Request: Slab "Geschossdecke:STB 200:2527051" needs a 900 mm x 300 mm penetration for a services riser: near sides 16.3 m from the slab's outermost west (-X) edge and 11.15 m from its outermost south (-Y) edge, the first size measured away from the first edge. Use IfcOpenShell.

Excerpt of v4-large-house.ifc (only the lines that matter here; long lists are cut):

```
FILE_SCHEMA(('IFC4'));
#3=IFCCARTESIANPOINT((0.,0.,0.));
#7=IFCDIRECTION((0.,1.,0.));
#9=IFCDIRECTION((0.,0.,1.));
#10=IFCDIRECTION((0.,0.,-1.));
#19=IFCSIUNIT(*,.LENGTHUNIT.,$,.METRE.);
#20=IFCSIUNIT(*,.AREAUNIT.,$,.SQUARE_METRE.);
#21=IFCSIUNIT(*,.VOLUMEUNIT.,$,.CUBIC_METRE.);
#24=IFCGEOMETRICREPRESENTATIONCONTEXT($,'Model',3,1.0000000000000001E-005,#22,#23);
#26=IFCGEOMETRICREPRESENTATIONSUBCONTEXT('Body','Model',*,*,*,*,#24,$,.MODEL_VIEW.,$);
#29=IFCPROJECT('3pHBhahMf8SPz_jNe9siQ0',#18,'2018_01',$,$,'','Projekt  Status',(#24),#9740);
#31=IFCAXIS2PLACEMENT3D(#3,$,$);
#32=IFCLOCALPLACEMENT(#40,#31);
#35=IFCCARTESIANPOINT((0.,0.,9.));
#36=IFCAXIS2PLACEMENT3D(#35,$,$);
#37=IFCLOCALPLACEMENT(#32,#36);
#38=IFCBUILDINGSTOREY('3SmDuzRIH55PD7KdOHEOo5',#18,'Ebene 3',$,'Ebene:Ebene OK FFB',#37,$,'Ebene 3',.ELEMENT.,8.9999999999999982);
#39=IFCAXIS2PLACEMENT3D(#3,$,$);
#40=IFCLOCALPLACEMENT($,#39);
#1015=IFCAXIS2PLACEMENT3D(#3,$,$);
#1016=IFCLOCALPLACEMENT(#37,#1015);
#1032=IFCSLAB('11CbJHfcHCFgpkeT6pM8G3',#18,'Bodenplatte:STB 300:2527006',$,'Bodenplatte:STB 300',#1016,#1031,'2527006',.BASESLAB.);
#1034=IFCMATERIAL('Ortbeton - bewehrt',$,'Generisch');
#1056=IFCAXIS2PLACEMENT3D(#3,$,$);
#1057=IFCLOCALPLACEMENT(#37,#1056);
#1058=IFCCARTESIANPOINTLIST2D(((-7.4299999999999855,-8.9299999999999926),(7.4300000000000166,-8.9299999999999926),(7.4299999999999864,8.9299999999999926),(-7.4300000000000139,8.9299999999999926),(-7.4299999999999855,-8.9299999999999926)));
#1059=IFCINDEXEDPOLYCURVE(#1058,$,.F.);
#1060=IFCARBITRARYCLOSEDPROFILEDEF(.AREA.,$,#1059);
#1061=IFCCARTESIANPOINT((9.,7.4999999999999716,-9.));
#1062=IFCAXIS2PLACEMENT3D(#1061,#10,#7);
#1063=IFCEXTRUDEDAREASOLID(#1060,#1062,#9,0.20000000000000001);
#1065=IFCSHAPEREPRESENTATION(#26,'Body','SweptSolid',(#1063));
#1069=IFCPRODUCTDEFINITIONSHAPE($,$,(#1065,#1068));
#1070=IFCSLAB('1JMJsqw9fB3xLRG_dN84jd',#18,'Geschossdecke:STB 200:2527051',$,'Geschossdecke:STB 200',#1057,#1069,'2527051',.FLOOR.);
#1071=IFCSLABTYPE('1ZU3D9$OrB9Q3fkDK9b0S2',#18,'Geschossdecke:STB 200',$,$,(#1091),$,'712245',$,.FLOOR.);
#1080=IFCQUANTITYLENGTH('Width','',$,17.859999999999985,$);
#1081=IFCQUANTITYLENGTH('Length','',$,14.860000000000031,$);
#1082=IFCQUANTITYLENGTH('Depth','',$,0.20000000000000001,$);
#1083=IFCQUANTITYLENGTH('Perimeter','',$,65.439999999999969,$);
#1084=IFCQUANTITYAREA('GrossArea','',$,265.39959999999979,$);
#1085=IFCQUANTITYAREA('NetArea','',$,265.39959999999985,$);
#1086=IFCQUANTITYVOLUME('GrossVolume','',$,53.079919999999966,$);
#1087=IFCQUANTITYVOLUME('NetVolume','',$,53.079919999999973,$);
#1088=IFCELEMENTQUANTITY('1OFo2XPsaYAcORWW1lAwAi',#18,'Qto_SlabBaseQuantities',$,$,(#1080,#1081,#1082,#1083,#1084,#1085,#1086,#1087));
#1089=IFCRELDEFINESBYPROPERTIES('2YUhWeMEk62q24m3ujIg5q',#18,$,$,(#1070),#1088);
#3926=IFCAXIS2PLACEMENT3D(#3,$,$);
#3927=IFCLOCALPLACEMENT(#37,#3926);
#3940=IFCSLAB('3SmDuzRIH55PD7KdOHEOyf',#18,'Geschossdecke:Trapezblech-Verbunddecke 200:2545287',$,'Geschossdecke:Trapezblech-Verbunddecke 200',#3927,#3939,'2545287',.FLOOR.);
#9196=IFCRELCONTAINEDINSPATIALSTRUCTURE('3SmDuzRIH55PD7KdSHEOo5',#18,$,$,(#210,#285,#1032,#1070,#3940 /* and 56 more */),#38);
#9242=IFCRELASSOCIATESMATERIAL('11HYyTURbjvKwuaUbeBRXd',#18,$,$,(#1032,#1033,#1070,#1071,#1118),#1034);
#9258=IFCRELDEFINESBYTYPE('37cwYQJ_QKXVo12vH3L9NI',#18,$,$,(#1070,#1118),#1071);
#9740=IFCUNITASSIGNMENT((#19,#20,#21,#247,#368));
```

```python
import numpy as np
import ifcopenshell
import ifcopenshell.api.feature
import ifcopenshell.api.geometry
import ifcopenshell.api.pset
import ifcopenshell.api.root
import ifcopenshell.geom
import ifcopenshell.util.element
import ifcopenshell.util.placement
import ifcopenshell.util.representation
import ifcopenshell.util.shape
import ifcopenshell.util.unit

model = ifcopenshell.open("v4-large-house.ifc")
unit_scale = ifcopenshell.util.unit.calculate_unit_scale(model)
area_scale = ifcopenshell.util.unit.calculate_unit_scale(model, "AREAUNIT")
volume_scale = ifcopenshell.util.unit.calculate_unit_scale(model, "VOLUMEUNIT")
settings = ifcopenshell.geom.settings()


def volume(element):
    """Net volume in cubic metres, openings subtracted."""
    shape = ifcopenshell.geom.create_shape(settings, element)
    return ifcopenshell.util.shape.get_volume(shape.geometry)


slab = model.by_guid("1JMJsqw9fB3xLRG_dN84jd")
before = volume(slab)

# Extent in the slab's own axes, in metres. The edges named are its -X and -Y sides.
slab_shape = ifcopenshell.geom.create_shape(settings, slab)
vertices = ifcopenshell.util.shape.get_vertices(slab_shape.geometry)
x_min, y_min, bottom = vertices.min(axis=0)
top = vertices[:, 2].max()

opening = ifcopenshell.api.root.create_entity(model, ifc_class="IfcOpeningElement", name="Services riser opening", predefined_type="OPENING")
context = ifcopenshell.util.representation.get_context(model, "Model", "Body", "MODEL_VIEW")
width, depth = 0.9, 0.3
outline = [(0.0, 0.0), (width, 0.0), (width, depth), (0.0, depth), (0.0, 0.0)]
# Overshoot both faces by 50 mm so the cut is clean.
shape = ifcopenshell.api.geometry.add_slab_representation(
    model, context=context, depth=top - bottom + 0.1, polyline=outline
)
ifcopenshell.api.geometry.assign_representation(model, product=opening, representation=shape)

matrix = ifcopenshell.util.placement.get_local_placement(slab.ObjectPlacement)
matrix[:, 3] = matrix @ np.append(np.array([x_min + 16.3, y_min + 11.15, bottom - 0.05]) / unit_scale, 1.0)
ifcopenshell.api.geometry.edit_object_placement(model, product=opening, matrix=matrix, is_si=False)
ifcopenshell.api.feature.add_feature(model, feature=opening, element=slab)

after = volume(slab)

# Update the slab's stored quantities.
qto = model.by_id(ifcopenshell.util.element.get_pset(slab, "Qto_SlabBaseQuantities", should_inherit=False)["id"])
ifcopenshell.api.pset.edit_qto(model, qto=qto, properties={
    "NetArea": after / (top - bottom) / area_scale,
    "NetVolume": after / volume_scale,
})

print(f"slab volume {before:.3f} -> {after:.3f} m3")

model.write("v4-large-house-out.ifc")
```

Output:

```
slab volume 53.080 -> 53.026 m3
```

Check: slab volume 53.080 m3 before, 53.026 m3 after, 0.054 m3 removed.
